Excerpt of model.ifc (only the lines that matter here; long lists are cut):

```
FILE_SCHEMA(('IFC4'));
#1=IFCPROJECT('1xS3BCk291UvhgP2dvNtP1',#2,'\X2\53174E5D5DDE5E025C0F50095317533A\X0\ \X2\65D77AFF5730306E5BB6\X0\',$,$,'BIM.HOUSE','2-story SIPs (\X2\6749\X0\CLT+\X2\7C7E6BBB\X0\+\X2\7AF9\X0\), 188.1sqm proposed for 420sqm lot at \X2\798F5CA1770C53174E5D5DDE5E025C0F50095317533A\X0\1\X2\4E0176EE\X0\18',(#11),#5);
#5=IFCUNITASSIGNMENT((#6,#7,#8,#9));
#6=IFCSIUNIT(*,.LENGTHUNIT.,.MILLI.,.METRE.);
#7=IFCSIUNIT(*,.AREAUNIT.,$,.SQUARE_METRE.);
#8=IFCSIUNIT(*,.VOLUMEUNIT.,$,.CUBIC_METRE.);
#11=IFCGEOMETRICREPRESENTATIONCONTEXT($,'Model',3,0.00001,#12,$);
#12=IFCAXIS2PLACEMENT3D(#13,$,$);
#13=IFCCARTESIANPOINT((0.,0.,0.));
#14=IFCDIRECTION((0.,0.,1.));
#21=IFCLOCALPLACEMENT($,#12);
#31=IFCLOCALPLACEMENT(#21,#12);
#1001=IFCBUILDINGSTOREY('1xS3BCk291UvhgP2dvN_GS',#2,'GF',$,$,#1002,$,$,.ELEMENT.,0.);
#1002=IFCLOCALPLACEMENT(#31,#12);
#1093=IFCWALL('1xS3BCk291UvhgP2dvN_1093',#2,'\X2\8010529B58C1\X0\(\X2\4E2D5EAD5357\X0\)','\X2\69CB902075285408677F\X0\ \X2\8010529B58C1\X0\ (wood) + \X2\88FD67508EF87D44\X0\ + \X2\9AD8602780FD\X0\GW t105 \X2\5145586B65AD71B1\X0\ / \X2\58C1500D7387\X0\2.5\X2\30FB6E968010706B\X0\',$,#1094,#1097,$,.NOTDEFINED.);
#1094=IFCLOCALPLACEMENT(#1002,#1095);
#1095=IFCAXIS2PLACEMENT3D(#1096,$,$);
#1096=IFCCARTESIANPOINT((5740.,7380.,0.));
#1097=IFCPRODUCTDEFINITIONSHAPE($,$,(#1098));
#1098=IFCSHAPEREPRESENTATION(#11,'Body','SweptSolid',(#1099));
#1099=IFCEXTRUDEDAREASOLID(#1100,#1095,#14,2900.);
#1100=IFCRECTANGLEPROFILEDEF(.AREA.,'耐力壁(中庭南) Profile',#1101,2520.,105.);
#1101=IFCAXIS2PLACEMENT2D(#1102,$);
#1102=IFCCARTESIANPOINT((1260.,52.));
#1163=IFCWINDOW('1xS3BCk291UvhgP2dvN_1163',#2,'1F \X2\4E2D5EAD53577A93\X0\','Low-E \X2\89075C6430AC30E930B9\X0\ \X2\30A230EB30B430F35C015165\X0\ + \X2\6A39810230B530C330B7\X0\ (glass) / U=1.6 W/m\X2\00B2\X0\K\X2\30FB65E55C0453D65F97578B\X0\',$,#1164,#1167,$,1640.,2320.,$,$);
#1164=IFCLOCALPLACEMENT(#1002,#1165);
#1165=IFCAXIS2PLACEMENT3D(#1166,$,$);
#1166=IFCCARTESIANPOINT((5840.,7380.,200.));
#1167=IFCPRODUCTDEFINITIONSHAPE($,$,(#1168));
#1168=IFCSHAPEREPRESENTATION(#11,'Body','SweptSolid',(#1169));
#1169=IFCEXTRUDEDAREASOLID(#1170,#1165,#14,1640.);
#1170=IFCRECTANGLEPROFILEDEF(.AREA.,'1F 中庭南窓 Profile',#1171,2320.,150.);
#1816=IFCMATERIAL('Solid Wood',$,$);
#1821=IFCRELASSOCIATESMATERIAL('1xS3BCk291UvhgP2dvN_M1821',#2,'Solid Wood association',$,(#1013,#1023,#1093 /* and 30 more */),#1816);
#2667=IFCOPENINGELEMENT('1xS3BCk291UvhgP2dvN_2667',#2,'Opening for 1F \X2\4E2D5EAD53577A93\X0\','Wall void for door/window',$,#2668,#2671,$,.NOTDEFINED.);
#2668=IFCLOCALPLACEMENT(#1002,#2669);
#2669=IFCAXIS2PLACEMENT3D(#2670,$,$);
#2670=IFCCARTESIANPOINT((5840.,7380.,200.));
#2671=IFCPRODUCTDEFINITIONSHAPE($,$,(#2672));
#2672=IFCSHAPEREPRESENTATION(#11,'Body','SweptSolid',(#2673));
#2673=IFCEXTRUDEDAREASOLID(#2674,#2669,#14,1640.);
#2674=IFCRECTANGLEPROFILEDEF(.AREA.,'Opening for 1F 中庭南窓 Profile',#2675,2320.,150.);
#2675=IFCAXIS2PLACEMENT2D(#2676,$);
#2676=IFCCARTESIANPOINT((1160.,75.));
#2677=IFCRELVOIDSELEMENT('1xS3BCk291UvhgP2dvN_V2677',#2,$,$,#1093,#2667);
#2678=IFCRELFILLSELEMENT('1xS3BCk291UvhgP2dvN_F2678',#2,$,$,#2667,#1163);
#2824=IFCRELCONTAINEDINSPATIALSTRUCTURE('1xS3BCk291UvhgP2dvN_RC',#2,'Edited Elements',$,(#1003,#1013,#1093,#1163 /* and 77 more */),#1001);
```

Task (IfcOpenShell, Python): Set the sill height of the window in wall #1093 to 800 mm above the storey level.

```python
import numpy as np
import ifcopenshell
import ifcopenshell.api.geometry
import ifcopenshell.geom
import ifcopenshell.util.element
import ifcopenshell.util.placement
import ifcopenshell.util.shape
import ifcopenshell.util.unit

model = ifcopenshell.open("model.ifc")
unit_scale = ifcopenshell.util.unit.calculate_unit_scale(model)

window = model.by_guid("1xS3BCk291UvhgP2dvN_1163")
opening = window.FillsVoids[0].RelatingOpeningElement
storey = ifcopenshell.util.element.get_container(window, ifc_class="IfcBuildingStorey")
level = ifcopenshell.util.placement.get_local_placement(storey.ObjectPlacement)[2, 3]

# The opening's origin need not be at the sill, so measure its lowest point.
shape = ifcopenshell.geom.create_shape(ifcopenshell.geom.settings(), opening)
bottom = ifcopenshell.util.shape.get_shape_bottom_elevation(shape, shape.geometry) / unit_scale
dz = level + 0.8 / unit_scale - bottom

shift = np.array([0.0, 0.0, dz])
# The window is not placed relative to its opening, so move both.
for product in (opening, window):
    matrix = ifcopenshell.util.placement.get_local_placement(product.ObjectPlacement)
    matrix[:3, 3] += shift
    ifcopenshell.api.geometry.edit_object_placement(model, product=product, matrix=matrix, is_si=False)

print(f"moved by {dz * unit_scale:+.3f} m")

model.write("model-out.ifc")
```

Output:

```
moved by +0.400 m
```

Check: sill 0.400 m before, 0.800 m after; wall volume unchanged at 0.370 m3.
